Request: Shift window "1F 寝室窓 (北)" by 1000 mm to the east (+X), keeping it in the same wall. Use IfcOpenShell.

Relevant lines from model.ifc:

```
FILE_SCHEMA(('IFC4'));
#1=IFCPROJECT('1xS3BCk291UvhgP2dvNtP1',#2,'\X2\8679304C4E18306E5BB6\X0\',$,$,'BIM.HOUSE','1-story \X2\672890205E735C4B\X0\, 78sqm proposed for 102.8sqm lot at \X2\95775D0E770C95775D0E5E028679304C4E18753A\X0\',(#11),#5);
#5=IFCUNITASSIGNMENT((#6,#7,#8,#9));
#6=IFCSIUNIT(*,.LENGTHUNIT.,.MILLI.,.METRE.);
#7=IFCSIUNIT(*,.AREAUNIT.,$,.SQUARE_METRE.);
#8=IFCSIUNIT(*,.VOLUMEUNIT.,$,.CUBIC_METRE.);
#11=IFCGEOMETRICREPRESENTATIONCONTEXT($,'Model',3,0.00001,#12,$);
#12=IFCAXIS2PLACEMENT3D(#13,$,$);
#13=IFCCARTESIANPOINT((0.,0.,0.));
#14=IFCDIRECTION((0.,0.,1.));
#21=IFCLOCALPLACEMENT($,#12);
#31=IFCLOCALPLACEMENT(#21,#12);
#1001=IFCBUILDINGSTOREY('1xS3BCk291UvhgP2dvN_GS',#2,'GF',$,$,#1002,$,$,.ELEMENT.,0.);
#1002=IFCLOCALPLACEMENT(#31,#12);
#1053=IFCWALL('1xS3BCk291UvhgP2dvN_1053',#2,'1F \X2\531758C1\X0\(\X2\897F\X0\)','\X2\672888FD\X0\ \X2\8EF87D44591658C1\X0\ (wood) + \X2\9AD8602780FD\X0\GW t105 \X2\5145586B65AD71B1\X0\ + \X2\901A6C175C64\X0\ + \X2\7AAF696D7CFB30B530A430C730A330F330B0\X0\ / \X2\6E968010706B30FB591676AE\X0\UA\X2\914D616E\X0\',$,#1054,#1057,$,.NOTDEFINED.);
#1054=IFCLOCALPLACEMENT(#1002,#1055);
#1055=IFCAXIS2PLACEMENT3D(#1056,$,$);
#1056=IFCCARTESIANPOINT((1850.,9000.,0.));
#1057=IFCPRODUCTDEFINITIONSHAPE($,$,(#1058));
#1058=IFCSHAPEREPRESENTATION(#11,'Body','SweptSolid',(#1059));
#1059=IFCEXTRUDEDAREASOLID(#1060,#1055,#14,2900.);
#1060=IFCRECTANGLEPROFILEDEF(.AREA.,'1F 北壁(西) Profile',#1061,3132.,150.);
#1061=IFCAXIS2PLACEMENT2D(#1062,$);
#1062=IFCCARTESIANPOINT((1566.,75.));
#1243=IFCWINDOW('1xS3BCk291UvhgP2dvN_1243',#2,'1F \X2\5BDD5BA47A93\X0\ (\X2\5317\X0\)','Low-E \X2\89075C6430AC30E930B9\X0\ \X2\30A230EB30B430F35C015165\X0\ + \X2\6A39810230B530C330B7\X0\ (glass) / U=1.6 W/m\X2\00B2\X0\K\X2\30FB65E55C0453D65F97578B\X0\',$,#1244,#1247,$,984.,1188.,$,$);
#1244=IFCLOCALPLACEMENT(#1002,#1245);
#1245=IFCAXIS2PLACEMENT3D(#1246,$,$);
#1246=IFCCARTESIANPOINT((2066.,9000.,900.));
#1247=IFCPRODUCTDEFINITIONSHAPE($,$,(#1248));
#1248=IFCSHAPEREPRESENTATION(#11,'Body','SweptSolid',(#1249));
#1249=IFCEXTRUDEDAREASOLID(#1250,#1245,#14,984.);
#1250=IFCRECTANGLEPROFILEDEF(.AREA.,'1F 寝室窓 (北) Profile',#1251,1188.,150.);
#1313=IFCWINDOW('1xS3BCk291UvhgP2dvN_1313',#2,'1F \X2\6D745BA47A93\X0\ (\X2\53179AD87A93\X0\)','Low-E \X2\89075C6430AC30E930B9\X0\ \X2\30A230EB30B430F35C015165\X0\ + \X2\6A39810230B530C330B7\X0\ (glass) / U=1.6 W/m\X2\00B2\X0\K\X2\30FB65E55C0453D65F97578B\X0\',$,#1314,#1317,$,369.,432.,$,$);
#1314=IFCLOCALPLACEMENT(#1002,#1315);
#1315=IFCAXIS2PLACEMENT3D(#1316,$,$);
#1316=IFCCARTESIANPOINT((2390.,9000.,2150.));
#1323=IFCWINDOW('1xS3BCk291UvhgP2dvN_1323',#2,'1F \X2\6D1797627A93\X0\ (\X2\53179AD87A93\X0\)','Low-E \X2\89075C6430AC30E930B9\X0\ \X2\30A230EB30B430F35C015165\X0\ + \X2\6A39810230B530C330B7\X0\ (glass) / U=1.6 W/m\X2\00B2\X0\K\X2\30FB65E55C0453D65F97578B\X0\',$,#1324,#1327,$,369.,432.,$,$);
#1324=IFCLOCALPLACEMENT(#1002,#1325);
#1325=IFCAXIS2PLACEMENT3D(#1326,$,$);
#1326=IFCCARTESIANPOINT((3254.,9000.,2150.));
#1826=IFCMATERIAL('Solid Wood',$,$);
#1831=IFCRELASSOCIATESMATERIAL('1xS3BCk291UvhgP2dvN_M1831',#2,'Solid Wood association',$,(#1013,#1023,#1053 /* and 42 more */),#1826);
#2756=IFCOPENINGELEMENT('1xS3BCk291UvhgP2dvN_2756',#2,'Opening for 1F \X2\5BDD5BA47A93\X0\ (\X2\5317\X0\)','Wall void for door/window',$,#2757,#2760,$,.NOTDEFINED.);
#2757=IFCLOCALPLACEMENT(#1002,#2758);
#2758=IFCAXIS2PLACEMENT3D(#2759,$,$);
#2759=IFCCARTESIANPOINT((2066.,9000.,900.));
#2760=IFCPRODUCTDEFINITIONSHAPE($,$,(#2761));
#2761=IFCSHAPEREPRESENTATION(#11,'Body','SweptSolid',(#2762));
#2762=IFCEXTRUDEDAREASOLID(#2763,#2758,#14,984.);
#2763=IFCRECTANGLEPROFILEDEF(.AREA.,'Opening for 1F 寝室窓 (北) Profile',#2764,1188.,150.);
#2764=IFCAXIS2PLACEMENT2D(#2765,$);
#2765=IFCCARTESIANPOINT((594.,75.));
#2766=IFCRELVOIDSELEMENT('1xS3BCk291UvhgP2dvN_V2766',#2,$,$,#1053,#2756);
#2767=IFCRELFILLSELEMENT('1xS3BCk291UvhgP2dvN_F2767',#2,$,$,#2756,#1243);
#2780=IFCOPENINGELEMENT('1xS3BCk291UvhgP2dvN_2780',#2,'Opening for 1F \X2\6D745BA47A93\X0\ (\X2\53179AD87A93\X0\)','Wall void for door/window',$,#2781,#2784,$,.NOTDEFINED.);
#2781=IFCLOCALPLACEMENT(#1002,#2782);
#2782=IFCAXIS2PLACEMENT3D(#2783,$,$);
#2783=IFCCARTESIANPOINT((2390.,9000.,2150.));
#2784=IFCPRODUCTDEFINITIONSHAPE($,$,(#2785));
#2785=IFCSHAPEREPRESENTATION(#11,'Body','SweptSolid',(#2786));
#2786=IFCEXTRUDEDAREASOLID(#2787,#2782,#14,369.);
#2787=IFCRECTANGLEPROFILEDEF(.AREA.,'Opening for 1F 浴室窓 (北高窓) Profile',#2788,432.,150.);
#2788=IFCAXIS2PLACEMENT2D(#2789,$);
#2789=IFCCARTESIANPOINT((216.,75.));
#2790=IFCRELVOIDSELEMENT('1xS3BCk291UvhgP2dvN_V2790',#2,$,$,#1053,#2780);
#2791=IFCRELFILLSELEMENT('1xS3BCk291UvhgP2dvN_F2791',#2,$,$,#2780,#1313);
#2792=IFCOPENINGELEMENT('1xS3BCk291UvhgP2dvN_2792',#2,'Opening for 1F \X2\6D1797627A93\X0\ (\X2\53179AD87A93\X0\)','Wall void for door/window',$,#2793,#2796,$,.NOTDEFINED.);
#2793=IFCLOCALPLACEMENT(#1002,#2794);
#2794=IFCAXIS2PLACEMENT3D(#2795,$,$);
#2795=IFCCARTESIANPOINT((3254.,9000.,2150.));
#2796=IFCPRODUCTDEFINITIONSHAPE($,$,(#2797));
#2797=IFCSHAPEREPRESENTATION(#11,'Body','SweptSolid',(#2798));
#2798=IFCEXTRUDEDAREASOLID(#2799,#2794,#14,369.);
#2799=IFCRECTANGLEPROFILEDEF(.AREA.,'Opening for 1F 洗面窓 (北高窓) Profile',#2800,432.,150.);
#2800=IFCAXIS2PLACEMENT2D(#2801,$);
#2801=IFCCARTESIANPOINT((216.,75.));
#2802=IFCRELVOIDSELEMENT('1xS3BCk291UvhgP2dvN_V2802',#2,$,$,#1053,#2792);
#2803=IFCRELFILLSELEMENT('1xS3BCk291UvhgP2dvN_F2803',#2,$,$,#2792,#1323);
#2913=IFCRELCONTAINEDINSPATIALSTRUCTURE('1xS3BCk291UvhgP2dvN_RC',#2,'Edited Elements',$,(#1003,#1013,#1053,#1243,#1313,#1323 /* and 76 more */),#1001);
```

```python
import ifcopenshell
import ifcopenshell.api.geometry
import ifcopenshell.util.placement

model = ifcopenshell.open("model.ifc")

window = model.by_guid("1xS3BCk291UvhgP2dvN_1243")
opening = window.FillsVoids[0].RelatingOpeningElement
wall = opening.VoidsElements[0].RelatingBuildingElement

wall_matrix = ifcopenshell.util.placement.get_local_placement(wall.ObjectPlacement)
shift = wall_matrix[:3, 0] * 1000.0
before = ifcopenshell.util.placement.get_local_placement(window.ObjectPlacement)[:3, 3].copy()

# The window is not placed relative to its opening, so move both.
for product in (opening, window):
    matrix = ifcopenshell.util.placement.get_local_placement(product.ObjectPlacement)
    matrix[:3, 3] += shift
    ifcopenshell.api.geometry.edit_object_placement(model, product=product, matrix=matrix, is_si=False)

after = ifcopenshell.util.placement.get_local_placement(window.ObjectPlacement)[:3, 3]
print("window moved by", (after - before).round(3) + 0.0)

model.write("model_updated.ifc")
```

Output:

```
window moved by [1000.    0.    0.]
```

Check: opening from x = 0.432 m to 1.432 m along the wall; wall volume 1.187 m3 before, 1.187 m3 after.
